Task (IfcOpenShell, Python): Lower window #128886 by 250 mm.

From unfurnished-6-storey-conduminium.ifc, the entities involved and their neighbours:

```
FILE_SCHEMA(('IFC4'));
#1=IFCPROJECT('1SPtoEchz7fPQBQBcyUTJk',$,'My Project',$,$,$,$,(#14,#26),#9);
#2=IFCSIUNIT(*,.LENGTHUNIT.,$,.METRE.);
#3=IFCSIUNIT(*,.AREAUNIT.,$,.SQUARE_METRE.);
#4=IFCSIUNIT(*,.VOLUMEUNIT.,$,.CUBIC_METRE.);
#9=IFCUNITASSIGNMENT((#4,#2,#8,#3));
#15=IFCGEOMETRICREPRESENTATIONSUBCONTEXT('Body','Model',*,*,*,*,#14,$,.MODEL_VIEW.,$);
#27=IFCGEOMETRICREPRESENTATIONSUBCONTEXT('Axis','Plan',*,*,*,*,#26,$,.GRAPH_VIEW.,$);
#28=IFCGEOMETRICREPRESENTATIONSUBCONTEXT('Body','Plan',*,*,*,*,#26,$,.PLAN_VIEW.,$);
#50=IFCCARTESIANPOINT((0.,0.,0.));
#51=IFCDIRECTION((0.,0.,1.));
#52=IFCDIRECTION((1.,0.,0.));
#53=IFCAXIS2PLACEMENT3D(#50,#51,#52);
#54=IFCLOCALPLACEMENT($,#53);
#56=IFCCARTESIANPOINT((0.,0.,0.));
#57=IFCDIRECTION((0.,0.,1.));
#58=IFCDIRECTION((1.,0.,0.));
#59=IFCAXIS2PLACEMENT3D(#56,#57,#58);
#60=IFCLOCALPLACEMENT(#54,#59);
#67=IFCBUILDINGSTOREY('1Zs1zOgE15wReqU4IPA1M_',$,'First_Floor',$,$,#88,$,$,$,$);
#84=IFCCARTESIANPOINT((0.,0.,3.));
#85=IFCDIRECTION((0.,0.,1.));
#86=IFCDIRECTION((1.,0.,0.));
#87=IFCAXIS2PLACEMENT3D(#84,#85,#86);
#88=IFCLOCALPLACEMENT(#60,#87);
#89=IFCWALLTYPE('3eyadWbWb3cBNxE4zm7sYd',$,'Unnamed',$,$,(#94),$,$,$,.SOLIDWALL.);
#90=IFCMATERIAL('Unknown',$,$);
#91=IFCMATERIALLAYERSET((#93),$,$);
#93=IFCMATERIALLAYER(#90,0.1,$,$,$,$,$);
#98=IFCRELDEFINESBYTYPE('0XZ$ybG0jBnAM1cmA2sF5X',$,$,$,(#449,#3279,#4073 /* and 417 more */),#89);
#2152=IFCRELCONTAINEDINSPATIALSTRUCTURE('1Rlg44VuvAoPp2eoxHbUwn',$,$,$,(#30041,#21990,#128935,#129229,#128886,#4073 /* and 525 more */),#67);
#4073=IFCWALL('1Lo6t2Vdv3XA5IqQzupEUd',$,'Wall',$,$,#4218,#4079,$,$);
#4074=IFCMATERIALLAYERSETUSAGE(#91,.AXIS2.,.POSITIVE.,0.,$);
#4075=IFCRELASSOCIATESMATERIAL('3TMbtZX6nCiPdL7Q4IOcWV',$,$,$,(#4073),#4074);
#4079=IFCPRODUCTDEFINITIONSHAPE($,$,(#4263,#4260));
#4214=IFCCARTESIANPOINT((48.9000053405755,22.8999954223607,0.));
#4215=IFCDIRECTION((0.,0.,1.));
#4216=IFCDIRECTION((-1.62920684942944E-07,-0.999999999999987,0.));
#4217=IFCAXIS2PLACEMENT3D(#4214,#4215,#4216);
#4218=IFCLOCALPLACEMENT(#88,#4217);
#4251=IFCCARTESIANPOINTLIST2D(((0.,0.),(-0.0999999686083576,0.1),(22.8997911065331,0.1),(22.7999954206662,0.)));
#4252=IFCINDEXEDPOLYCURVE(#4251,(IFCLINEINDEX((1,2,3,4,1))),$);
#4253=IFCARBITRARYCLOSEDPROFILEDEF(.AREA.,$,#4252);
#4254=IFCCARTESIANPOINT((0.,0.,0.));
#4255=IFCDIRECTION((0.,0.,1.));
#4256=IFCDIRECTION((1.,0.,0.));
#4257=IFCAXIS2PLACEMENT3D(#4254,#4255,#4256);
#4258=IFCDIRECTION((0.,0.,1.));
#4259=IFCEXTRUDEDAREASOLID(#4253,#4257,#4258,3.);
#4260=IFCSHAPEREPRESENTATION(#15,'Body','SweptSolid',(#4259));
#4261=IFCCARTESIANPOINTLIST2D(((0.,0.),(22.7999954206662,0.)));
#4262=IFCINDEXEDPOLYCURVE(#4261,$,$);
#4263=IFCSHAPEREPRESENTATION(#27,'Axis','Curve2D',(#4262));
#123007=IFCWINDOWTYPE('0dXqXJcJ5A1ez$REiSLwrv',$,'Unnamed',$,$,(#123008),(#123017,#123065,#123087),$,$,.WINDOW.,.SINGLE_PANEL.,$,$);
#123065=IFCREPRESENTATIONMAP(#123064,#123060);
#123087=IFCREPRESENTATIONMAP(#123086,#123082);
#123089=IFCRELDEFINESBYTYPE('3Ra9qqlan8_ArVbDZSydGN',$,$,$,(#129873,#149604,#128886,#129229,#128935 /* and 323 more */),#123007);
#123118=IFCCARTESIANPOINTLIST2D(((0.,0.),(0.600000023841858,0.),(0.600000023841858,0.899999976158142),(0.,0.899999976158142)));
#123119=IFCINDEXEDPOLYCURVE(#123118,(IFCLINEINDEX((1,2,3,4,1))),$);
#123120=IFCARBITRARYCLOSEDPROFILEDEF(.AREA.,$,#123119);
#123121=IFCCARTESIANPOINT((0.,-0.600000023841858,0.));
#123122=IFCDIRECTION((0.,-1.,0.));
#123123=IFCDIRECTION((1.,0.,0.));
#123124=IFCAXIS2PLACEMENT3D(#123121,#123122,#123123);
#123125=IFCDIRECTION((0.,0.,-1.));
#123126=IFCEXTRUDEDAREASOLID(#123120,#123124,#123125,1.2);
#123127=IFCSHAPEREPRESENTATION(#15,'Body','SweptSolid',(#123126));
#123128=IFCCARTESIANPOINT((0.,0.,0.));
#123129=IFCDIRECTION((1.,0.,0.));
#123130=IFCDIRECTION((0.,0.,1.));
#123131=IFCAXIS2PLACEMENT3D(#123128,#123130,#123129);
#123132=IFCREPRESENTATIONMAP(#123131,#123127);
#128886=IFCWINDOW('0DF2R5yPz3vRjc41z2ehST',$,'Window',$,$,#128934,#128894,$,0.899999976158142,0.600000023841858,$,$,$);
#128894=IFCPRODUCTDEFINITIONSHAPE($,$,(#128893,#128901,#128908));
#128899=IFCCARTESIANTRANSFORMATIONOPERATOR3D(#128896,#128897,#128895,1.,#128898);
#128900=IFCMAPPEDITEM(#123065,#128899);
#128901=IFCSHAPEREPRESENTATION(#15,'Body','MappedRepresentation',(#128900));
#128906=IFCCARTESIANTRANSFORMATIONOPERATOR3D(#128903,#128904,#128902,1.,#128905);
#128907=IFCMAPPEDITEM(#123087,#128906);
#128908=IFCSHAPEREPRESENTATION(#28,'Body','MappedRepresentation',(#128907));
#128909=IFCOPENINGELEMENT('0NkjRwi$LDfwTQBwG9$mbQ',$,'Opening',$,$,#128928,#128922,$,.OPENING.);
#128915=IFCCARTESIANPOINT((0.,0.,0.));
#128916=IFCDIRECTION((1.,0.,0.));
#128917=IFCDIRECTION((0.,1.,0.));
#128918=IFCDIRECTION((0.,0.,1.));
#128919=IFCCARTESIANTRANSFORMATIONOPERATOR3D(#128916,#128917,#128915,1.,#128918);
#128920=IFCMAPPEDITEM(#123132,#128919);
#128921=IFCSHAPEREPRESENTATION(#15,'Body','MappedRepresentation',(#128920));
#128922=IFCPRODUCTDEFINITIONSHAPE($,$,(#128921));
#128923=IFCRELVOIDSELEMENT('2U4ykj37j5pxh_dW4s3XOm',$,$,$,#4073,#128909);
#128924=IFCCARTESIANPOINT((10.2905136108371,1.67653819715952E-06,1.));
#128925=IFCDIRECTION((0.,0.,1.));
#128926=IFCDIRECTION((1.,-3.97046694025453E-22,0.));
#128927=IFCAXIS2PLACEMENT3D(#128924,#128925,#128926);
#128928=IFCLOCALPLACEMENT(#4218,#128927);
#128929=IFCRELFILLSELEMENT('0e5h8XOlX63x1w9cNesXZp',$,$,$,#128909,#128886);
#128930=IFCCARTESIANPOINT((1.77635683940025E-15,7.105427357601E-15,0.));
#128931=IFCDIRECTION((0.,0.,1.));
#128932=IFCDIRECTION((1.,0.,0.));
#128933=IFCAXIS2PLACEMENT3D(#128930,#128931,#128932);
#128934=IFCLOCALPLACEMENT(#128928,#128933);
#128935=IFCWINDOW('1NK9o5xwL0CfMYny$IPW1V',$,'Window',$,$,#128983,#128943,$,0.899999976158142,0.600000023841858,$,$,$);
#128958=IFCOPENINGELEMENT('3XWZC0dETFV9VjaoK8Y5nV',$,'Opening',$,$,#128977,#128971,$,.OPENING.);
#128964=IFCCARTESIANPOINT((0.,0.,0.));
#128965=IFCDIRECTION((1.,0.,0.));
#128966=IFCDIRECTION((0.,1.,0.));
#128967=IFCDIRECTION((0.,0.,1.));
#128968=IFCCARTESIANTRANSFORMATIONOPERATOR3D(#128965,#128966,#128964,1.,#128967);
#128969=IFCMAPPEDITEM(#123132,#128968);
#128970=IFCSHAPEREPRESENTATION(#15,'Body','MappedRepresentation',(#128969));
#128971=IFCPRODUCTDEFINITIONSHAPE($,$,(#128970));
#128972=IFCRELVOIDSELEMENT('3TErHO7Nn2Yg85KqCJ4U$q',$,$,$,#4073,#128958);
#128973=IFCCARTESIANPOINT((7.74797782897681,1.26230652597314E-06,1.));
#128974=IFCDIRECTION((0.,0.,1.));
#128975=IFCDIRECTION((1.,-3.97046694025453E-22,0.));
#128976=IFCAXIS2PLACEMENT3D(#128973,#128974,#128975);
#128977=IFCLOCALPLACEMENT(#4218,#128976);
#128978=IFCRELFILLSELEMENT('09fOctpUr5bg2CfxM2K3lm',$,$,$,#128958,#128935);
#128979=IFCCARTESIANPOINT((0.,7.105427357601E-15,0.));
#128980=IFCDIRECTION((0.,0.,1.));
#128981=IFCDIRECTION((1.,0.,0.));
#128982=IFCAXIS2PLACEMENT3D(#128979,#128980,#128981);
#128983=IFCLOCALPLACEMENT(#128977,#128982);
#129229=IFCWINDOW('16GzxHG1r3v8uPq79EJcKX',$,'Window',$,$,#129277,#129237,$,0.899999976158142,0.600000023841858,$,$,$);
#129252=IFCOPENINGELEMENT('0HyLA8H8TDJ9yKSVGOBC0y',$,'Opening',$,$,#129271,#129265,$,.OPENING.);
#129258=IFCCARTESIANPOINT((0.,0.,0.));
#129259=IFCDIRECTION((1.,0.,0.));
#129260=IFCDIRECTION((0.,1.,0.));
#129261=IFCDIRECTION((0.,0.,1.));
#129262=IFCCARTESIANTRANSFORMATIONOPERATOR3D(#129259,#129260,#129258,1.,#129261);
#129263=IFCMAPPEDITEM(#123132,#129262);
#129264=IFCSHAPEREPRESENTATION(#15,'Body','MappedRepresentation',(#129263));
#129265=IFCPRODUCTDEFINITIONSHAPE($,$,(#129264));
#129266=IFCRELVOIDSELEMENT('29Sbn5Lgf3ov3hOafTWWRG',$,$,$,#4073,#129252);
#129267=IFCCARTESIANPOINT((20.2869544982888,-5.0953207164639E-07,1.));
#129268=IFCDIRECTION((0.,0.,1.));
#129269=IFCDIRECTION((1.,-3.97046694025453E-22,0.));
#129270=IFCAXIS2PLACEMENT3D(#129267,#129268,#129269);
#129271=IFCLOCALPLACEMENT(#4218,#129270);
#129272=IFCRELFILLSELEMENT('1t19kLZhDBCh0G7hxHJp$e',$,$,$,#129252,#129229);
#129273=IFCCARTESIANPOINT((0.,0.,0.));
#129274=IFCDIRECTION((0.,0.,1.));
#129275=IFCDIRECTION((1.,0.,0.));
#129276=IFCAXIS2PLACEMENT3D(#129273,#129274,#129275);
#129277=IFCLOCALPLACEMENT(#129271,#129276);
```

```python
import numpy as np
import ifcopenshell
import ifcopenshell.api.geometry
import ifcopenshell.util.placement
import ifcopenshell.util.unit

model = ifcopenshell.open("unfurnished-6-storey-conduminium.ifc")
unit_scale = ifcopenshell.util.unit.calculate_unit_scale(model)

window = model.by_guid("0DF2R5yPz3vRjc41z2ehST")
opening = window.FillsVoids[0].RelatingOpeningElement
dz = -0.25 / unit_scale

shift = np.array([0.0, 0.0, dz])
# The window is placed relative to its opening, so it follows when the opening moves.
matrix = ifcopenshell.util.placement.get_local_placement(opening.ObjectPlacement)
matrix[:3, 3] += shift
ifcopenshell.api.geometry.edit_object_placement(
    model, product=opening, matrix=matrix, is_si=False, should_transform_children=True
)

print(f"moved by {dz * unit_scale:+.3f} m")

model.write("unfurnished-6-storey-conduminium-out.ifc")
```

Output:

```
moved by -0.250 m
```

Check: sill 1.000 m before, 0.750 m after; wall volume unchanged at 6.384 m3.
